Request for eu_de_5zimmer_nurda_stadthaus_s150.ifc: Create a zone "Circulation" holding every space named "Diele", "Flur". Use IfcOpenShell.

First a look at what the model holds.

```python
import ifcopenshell

model = ifcopenshell.open("eu_de_5zimmer_nurda_stadthaus_s150.ifc")
print(model.schema)
seen = {}
for space in model.by_type("IfcSpace"):
    seen[space.LongName] = seen.get(space.LongName, 0) + 1
for name, count in sorted(seen.items(), key=str):
    print(count, "x", name)
print("zones:", [z.Name for z in model.by_type("IfcZone")][:20])
```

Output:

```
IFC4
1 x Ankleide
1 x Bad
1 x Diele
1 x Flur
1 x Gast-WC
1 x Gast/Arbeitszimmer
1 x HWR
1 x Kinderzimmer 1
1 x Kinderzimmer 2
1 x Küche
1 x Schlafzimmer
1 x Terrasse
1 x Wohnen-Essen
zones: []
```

```python
import ifcopenshell
import ifcopenshell.api.group
import ifcopenshell.api.root

model = ifcopenshell.open("eu_de_5zimmer_nurda_stadthaus_s150.ifc")

names = {"Diele", "Flur"}
spaces = [s for s in model.by_type("IfcSpace") if s.LongName in names]

zone = ifcopenshell.api.root.create_entity(model, ifc_class="IfcZone", name="Circulation")
ifcopenshell.api.group.assign_group(model, products=spaces, group=zone)
print(len(spaces), "spaces in", zone.Name)

model.write("eu_de_5zimmer_nurda_stadthaus_s150_rev.ifc")
```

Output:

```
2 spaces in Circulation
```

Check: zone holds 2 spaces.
